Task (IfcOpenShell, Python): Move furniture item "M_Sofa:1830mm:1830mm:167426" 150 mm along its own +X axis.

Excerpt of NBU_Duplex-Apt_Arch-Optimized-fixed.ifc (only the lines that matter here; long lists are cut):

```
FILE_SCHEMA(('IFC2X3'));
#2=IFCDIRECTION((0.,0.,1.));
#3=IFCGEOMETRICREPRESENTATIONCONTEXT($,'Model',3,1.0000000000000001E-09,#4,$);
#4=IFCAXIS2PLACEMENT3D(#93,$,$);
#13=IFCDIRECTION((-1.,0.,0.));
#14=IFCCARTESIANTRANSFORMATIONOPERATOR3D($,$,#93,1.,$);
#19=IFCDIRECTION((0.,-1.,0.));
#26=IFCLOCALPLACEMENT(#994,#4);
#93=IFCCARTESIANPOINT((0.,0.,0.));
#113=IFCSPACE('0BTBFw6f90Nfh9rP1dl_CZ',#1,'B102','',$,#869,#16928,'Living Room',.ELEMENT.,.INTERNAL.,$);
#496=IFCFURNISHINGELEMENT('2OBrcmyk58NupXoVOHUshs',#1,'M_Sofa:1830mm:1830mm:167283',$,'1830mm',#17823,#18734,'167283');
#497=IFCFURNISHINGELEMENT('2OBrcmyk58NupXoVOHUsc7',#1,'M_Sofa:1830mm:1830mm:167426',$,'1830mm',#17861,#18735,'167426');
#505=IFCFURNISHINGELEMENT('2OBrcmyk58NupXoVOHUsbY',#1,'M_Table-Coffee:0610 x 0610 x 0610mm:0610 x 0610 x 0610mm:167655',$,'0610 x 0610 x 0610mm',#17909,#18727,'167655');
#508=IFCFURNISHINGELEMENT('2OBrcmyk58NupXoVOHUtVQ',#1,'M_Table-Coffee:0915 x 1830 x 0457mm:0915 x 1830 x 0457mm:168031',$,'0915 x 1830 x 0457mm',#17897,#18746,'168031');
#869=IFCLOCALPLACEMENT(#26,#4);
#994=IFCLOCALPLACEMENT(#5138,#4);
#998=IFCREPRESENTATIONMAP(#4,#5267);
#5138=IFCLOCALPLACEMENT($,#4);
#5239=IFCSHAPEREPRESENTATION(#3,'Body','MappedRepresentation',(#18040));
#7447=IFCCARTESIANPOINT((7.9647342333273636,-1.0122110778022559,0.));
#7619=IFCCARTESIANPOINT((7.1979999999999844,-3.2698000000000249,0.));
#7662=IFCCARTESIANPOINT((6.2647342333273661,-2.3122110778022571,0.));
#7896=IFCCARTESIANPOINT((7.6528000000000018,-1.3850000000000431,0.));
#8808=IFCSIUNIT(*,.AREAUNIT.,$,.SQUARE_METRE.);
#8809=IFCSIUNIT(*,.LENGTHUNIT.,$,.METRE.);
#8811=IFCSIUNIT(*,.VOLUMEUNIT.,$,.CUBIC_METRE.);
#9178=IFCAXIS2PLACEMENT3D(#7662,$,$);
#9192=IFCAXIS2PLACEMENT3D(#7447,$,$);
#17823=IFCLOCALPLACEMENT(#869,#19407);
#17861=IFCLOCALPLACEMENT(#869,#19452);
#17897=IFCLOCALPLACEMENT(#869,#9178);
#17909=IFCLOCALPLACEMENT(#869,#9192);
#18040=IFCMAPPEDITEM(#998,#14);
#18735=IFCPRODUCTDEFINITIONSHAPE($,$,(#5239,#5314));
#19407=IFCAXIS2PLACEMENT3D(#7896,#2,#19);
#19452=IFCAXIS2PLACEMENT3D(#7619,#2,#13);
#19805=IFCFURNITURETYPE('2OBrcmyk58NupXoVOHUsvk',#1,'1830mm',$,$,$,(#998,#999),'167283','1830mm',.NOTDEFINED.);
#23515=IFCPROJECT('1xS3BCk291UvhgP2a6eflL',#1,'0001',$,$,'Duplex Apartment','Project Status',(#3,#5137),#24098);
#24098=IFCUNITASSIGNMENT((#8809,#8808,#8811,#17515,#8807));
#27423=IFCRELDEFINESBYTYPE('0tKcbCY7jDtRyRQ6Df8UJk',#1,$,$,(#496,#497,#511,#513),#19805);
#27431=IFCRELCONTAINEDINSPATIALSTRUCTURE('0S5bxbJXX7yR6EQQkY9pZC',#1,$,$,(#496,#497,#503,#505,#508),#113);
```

```python
import ifcopenshell
import ifcopenshell.api.geometry
import ifcopenshell.util.placement
import ifcopenshell.util.unit

model = ifcopenshell.open("NBU_Duplex-Apt_Arch-Optimized-fixed.ifc")
unit_scale = ifcopenshell.util.unit.calculate_unit_scale(model)

item = model.by_id(497)
matrix = ifcopenshell.util.placement.get_local_placement(item.ObjectPlacement)
matrix[:3, 3] += matrix[:3, 0] * 0.15 / unit_scale
ifcopenshell.api.geometry.edit_object_placement(model, product=item, matrix=matrix, is_si=False)

print(ifcopenshell.util.placement.get_local_placement(item.ObjectPlacement).round(3) + 0.0)

model.write("NBU_Duplex-Apt_Arch-Optimized-fixed_updated.ifc")
```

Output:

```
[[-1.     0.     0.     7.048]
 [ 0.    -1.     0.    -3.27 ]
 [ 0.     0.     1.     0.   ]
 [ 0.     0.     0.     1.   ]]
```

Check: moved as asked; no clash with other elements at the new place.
